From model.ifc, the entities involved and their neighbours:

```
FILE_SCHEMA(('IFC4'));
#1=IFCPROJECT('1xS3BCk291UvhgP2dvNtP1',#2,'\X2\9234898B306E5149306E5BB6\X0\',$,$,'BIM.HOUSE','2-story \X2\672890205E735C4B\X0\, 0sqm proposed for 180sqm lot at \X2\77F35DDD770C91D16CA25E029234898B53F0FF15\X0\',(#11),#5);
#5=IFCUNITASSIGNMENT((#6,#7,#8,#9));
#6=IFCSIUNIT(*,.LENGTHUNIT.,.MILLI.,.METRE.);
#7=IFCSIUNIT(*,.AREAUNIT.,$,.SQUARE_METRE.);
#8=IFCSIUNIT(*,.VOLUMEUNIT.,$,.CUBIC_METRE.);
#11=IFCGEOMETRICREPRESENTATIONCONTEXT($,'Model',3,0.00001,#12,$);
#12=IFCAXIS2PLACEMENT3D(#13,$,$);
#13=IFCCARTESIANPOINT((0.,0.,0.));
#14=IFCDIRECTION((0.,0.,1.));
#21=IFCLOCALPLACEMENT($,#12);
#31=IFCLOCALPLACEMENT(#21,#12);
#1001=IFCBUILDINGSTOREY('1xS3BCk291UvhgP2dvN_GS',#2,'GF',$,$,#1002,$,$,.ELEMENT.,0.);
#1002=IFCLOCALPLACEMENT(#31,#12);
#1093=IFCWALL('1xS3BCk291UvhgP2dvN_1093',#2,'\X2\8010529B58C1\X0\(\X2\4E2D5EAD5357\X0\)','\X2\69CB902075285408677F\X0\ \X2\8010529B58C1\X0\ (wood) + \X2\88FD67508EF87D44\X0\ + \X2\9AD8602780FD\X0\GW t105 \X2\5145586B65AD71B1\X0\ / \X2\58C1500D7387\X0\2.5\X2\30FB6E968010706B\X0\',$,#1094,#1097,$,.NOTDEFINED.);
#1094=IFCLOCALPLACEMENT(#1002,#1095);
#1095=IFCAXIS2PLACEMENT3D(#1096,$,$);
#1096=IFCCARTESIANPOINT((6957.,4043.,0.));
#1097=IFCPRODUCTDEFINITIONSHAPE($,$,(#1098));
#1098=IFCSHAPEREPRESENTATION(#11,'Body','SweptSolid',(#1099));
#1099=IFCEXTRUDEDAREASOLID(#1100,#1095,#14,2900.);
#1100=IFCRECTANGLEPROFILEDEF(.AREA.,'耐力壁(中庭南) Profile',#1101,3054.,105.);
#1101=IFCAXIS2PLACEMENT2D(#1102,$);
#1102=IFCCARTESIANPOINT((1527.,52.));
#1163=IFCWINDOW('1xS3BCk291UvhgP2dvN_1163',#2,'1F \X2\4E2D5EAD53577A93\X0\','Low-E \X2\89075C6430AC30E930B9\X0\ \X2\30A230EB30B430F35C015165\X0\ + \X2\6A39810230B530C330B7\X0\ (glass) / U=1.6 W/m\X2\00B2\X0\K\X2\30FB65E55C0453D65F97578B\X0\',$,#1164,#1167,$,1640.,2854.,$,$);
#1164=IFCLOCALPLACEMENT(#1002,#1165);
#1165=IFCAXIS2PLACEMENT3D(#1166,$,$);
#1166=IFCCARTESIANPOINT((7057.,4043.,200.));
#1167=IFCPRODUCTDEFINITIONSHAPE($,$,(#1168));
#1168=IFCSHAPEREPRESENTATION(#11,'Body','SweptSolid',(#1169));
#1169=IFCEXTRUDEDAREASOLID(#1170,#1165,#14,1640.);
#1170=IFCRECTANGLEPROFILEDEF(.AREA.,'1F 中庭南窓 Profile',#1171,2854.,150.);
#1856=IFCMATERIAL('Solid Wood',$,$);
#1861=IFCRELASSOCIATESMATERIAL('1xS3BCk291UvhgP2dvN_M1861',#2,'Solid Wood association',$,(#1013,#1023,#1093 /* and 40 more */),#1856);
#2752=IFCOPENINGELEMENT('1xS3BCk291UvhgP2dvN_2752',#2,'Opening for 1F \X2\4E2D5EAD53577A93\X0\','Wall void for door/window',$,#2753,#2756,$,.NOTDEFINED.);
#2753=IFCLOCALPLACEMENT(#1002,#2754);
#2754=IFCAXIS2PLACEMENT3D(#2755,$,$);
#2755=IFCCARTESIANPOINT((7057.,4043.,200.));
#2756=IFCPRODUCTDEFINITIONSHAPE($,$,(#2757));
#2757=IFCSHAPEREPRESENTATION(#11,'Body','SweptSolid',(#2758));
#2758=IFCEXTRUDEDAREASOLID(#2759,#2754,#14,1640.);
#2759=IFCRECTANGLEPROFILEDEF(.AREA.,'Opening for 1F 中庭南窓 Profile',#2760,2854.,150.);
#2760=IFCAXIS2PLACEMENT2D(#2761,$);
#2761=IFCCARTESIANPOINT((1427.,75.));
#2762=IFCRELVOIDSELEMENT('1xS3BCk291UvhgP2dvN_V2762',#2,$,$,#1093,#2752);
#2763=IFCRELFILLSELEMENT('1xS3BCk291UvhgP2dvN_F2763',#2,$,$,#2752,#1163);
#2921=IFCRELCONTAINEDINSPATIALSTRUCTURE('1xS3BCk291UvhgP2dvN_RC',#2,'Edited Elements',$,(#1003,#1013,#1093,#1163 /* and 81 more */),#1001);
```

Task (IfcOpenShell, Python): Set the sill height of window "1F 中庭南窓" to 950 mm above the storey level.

```python
import numpy as np
import ifcopenshell
import ifcopenshell.api.geometry
import ifcopenshell.geom
import ifcopenshell.util.element
import ifcopenshell.util.placement
import ifcopenshell.util.shape
import ifcopenshell.util.unit

model = ifcopenshell.open("model.ifc")
unit_scale = ifcopenshell.util.unit.calculate_unit_scale(model)

window = model.by_guid("1xS3BCk291UvhgP2dvN_1163")
opening = window.FillsVoids[0].RelatingOpeningElement
storey = ifcopenshell.util.element.get_container(window, ifc_class="IfcBuildingStorey")
level = ifcopenshell.util.placement.get_local_placement(storey.ObjectPlacement)[2, 3]

# The opening's origin need not be at the sill, so measure its lowest point.
shape = ifcopenshell.geom.create_shape(ifcopenshell.geom.settings(), opening)
bottom = ifcopenshell.util.shape.get_shape_bottom_elevation(shape, shape.geometry) / unit_scale
dz = level + 950.0 - bottom

shift = np.array([0.0, 0.0, dz])
# The window is not placed relative to its opening, so move both.
for product in (opening, window):
    matrix = ifcopenshell.util.placement.get_local_placement(product.ObjectPlacement)
    matrix[:3, 3] += shift
    ifcopenshell.api.geometry.edit_object_placement(model, product=product, matrix=matrix, is_si=False)

print(f"moved by {dz * unit_scale:+.3f} m")

model.write("model_updated.ifc")
```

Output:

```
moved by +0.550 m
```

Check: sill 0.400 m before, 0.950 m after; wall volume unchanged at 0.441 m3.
